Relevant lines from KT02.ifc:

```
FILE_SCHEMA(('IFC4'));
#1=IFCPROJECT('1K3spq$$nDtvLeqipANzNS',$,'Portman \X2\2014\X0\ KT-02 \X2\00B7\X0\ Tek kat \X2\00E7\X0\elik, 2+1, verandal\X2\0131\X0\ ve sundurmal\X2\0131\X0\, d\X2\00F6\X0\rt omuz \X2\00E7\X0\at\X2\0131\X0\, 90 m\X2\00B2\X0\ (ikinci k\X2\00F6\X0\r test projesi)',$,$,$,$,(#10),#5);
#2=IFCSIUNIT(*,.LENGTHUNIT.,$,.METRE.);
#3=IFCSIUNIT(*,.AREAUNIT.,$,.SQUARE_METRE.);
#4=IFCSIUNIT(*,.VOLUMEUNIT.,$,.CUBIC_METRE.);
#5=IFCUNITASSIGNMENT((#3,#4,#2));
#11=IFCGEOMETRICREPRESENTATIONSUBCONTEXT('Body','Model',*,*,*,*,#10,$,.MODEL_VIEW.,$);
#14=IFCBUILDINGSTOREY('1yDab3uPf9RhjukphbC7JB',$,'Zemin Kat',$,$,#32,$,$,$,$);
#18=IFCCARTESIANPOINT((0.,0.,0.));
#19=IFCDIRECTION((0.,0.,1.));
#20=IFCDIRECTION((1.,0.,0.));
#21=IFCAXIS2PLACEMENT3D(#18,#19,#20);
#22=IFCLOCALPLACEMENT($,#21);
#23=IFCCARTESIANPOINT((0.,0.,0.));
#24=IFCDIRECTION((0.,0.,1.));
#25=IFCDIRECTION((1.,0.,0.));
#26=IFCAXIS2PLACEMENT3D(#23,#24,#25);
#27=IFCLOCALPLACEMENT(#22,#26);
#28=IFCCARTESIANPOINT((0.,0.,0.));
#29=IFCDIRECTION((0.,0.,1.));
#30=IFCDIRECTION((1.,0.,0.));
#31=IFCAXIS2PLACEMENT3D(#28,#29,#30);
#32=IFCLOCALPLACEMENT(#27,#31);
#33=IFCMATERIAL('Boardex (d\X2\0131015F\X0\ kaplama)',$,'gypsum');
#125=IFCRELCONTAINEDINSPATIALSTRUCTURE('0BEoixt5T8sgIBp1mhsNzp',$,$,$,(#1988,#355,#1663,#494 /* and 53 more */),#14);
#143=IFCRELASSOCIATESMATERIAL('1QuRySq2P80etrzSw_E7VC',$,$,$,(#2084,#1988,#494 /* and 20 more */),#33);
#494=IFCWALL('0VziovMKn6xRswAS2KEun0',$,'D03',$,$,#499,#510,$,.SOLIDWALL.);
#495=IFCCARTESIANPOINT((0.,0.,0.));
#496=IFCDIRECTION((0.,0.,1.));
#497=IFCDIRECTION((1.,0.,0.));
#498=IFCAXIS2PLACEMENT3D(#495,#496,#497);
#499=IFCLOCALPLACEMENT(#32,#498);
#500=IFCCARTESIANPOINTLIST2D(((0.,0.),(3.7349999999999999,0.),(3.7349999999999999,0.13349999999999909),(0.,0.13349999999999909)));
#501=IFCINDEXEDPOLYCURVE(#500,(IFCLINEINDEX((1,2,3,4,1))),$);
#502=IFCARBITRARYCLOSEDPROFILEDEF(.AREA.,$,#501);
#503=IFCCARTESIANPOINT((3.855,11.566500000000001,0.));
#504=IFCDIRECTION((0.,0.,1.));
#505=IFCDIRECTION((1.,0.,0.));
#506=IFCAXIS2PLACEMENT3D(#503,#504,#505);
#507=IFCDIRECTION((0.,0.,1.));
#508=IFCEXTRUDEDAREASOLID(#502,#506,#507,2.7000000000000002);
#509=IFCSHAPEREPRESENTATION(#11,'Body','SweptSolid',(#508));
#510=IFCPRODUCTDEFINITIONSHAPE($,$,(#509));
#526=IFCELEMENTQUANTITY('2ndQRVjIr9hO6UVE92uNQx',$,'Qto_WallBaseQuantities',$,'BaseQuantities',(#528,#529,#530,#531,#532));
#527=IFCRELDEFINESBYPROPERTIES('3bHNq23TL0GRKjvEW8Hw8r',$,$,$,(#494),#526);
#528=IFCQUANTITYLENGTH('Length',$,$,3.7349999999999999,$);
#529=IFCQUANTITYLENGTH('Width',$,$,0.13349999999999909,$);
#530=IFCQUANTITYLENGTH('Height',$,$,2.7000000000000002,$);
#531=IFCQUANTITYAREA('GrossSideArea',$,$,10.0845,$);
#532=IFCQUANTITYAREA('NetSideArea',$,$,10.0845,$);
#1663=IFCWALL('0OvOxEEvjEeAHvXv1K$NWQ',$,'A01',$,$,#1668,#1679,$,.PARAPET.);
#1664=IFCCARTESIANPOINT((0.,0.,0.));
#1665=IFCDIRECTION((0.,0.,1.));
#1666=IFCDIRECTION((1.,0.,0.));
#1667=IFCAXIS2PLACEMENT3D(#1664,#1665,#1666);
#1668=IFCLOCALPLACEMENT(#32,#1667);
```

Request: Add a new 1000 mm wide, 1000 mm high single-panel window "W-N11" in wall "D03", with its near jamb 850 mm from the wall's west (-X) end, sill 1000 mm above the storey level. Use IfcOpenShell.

```python
import numpy as np
import ifcopenshell
import ifcopenshell.api.feature
import ifcopenshell.api.geometry
import ifcopenshell.api.pset
import ifcopenshell.api.root
import ifcopenshell.api.spatial
import ifcopenshell.geom
import ifcopenshell.util.element
import ifcopenshell.util.placement
import ifcopenshell.util.representation
import ifcopenshell.util.shape
import ifcopenshell.util.unit

model = ifcopenshell.open("KT02.ifc")
unit_scale = ifcopenshell.util.unit.calculate_unit_scale(model)
area_scale = ifcopenshell.util.unit.calculate_unit_scale(model, "AREAUNIT")
settings = ifcopenshell.geom.settings()


def volume(element):
    """Net volume in cubic metres, openings subtracted."""
    shape = ifcopenshell.geom.create_shape(settings, element)
    return ifcopenshell.util.shape.get_volume(shape.geometry)


wall = model.by_id(494)
storey = ifcopenshell.util.element.get_container(wall, ifc_class="IfcBuildingStorey")
context = ifcopenshell.util.representation.get_context(model, "Model", "Body", "MODEL_VIEW")
before = volume(wall)

width, height, from_end, sill = 1, 1, 0.85, 1  # metres

# The wall runs along its own X axis, and the end named is its -X end.
wall_shape = ifcopenshell.geom.create_shape(settings, wall)
x, y, z = ifcopenshell.util.shape.get_vertices(wall_shape.geometry).T
start = x.min() + from_end
face, thickness = float(y.min()), float(y.max() - y.min())
wall_matrix = ifcopenshell.util.placement.get_local_placement(wall.ObjectPlacement)
level = ifcopenshell.util.placement.get_local_placement(storey.ObjectPlacement)[2, 3]


def in_wall(x, y):
    """Placement at x, y metres in the wall's axes, at sill height."""
    matrix = wall_matrix.copy()
    matrix[:, 3] = wall_matrix @ np.array([x / unit_scale, y / unit_scale, 0.0, 1.0])
    matrix[2, 3] = level + sill / unit_scale
    return matrix


# Opening: a box that overshoots both wall faces by 50 mm.
opening = ifcopenshell.api.root.create_entity(model, ifc_class="IfcOpeningElement", predefined_type="OPENING")
box = ifcopenshell.api.geometry.add_wall_representation(
    model, context=context, length=width, height=height, thickness=thickness + 0.1
)
ifcopenshell.api.geometry.assign_representation(model, product=opening, representation=box)
ifcopenshell.api.geometry.edit_object_placement(model, product=opening, matrix=in_wall(start, face - 0.05), is_si=False)
ifcopenshell.api.feature.add_feature(model, feature=opening, element=wall)

window = ifcopenshell.api.root.create_entity(model, ifc_class="IfcWindow", name="W-N11", predefined_type="WINDOW")
window.OverallWidth, window.OverallHeight = width / unit_scale, height / unit_scale
window.PartitioningType = "SINGLE_PANEL"
body = ifcopenshell.api.geometry.add_window_representation(
    model,
    context=context,
    overall_width=window.OverallWidth,
    overall_height=window.OverallHeight,
    partition_type="SINGLE_PANEL",
)
ifcopenshell.api.geometry.assign_representation(model, product=window, representation=body)
ifcopenshell.api.spatial.assign_container(model, products=[window], relating_structure=storey)
ifcopenshell.api.feature.add_filling(model, opening=opening, element=window)

# Centre the window in the wall's thickness.
ifcopenshell.api.geometry.edit_object_placement(model, product=window, matrix=in_wall(start, face), is_si=False)
window_shape = ifcopenshell.geom.create_shape(settings, window)
depth = ifcopenshell.util.shape.get_vertices(window_shape.geometry)[:, 1]
offset = face + thickness / 2 - (depth.min() + depth.max()) / 2
ifcopenshell.api.geometry.edit_object_placement(model, product=window, matrix=in_wall(start, offset), is_si=False)

after = volume(wall)

# Update the wall's stored quantities.
qto = model.by_id(ifcopenshell.util.element.get_pset(wall, "Qto_WallBaseQuantities", should_inherit=False)["id"])
ifcopenshell.api.pset.edit_qto(model, qto=qto, properties={"NetSideArea": after / thickness / area_scale})

print(f"wall volume {before:.3f} -> {after:.3f} m3")

model.write("KT02_rev.ifc")
```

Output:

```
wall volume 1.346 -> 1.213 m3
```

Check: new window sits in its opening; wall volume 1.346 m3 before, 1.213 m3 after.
